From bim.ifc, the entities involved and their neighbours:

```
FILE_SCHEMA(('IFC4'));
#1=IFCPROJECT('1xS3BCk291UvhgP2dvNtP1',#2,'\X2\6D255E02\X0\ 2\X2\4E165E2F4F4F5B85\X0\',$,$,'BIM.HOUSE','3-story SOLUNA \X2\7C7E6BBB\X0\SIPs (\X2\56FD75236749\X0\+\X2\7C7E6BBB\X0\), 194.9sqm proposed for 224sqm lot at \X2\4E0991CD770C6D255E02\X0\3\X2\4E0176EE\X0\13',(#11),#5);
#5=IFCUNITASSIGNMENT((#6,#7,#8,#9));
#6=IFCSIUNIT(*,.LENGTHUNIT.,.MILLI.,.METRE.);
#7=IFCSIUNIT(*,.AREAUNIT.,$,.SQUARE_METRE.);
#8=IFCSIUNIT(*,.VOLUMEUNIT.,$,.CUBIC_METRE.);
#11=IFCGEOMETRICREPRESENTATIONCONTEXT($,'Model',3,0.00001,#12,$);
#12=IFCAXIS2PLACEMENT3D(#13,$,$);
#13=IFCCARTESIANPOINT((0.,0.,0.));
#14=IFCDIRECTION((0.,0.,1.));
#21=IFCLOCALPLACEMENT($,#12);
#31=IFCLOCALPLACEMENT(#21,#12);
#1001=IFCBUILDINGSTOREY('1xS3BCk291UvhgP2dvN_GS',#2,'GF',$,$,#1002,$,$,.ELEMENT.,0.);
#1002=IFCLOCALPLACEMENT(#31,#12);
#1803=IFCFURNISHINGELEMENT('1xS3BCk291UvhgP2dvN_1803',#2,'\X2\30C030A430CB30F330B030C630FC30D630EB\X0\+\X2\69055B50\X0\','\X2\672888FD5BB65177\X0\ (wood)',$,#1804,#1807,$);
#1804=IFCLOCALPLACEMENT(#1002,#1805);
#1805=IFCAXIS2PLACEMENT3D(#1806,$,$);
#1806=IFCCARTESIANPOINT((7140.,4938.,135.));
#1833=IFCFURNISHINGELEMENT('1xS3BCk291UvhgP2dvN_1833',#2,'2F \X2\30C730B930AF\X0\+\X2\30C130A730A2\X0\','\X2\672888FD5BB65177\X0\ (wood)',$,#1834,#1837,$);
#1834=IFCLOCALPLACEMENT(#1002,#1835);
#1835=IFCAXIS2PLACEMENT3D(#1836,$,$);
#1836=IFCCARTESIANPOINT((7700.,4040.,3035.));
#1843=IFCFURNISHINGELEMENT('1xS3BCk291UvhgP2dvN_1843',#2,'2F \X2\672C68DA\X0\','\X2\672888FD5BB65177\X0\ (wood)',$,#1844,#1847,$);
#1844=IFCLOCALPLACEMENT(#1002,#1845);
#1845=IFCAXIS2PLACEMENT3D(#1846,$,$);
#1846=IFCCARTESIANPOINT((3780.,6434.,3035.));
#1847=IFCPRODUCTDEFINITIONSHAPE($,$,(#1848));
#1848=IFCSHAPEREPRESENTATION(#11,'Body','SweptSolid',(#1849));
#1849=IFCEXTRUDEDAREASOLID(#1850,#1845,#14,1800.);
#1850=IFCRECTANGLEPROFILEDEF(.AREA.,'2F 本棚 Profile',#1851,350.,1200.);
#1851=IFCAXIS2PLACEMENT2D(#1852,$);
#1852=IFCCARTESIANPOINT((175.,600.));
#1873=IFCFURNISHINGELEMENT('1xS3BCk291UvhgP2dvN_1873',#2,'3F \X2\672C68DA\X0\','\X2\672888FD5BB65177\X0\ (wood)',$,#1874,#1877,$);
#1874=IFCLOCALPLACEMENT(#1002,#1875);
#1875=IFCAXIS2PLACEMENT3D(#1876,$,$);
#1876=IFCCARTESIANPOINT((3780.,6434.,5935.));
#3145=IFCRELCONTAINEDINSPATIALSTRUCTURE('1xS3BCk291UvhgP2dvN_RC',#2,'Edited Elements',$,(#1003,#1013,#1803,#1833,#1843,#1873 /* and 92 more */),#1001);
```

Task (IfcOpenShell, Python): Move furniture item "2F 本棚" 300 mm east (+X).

```python
import ifcopenshell
import ifcopenshell.api.geometry
import ifcopenshell.util.placement
import ifcopenshell.util.unit

model = ifcopenshell.open("bim.ifc")
unit_scale = ifcopenshell.util.unit.calculate_unit_scale(model)

item = model.by_guid("1xS3BCk291UvhgP2dvN_1843")
matrix = ifcopenshell.util.placement.get_local_placement(item.ObjectPlacement)
matrix[0, 3] += 0.3 / unit_scale
ifcopenshell.api.geometry.edit_object_placement(model, product=item, matrix=matrix, is_si=False)

print(ifcopenshell.util.placement.get_local_placement(item.ObjectPlacement).round(3) + 0.0)

model.write("bim-out.ifc")
```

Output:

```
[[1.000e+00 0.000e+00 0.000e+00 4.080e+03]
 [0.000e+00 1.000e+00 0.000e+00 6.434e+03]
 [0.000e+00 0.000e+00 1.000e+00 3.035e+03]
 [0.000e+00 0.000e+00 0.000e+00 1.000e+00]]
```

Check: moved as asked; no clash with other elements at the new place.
